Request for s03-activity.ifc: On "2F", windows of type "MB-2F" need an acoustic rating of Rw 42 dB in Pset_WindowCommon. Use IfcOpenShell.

First a look at what the model holds.

```python
import ifcopenshell
import ifcopenshell.util.element

model = ifcopenshell.open("s03-activity.ifc")
print(model.schema)
storey = next(s for s in model.by_type("IfcBuildingStorey") if s.Name == "2F")
windows = [e for e in ifcopenshell.util.element.get_decomposition(storey) if e.is_a("IfcWindow")]
seen = {}
for e in windows:
    element_type = ifcopenshell.util.element.get_type(e)
    key = (element_type.Name if element_type != e and element_type else None, ifcopenshell.util.element.get_pset(e, "Pset_WindowCommon", "AcousticRating"))
    seen[key] = seen.get(key, 0) + 1
for (name, value), count in sorted(seen.items(), key=str):
    print(count, "x", name, "|", value)
```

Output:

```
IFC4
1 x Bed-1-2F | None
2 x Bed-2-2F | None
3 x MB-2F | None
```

```python
import ifcopenshell
import ifcopenshell.api.pset
import ifcopenshell.util.element

model = ifcopenshell.open("s03-activity.ifc")

storey = next(s for s in model.by_type("IfcBuildingStorey") if s.Name == "2F")
windows = [e for e in ifcopenshell.util.element.get_decomposition(storey) if e.is_a("IfcWindow")]

count = 0
for e in windows:
    element_type = ifcopenshell.util.element.get_type(e)
    if element_type in (None, e) or element_type.Name != "MB-2F":
        continue
    # add_pset returns the element's existing set when there is one.
    pset = ifcopenshell.api.pset.add_pset(model, product=e, name="Pset_WindowCommon")
    ifcopenshell.api.pset.edit_pset(model, pset=pset, properties={"AcousticRating": "Rw 42 dB"})
    count += 1

print(count, "windows updated")

model.write("s03-activity_v2.ifc")
```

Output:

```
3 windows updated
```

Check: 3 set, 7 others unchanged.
